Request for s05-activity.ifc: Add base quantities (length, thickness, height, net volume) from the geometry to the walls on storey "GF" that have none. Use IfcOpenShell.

First a look at what the model holds.

```python
import ifcopenshell
import ifcopenshell.util.element
import ifcopenshell.util.unit

model = ifcopenshell.open("s05-activity.ifc")
print(model.schema)
for unit_type in ("LENGTHUNIT", "AREAUNIT", "VOLUMEUNIT"):
    print(unit_type, ifcopenshell.util.unit.calculate_unit_scale(model, unit_type))
storey = next(s for s in model.by_type("IfcBuildingStorey") if s.Name == "GF")
walls = [e for e in ifcopenshell.util.element.get_decomposition(storey) if e.is_a("IfcWall")]
for e in sorted(walls, key=lambda e: e.id()):
    print(e.id(), e.is_a(), e.Name, list(ifcopenshell.util.element.get_psets(e, qtos_only=True)), sep=" | ")
```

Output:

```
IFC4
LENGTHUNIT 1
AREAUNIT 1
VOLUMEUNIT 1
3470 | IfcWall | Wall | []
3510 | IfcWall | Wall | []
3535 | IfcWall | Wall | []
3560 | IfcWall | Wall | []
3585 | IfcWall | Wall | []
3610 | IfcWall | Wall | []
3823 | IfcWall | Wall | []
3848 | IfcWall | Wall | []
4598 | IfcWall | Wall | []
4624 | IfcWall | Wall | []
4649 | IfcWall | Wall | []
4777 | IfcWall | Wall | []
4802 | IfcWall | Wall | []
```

```python
import ifcopenshell
import ifcopenshell.api.pset
import ifcopenshell.geom
import ifcopenshell.util.element
import ifcopenshell.util.shape
import ifcopenshell.util.unit

model = ifcopenshell.open("s05-activity.ifc")
unit_scale = ifcopenshell.util.unit.calculate_unit_scale(model)
volume_scale = ifcopenshell.util.unit.calculate_unit_scale(model, "VOLUMEUNIT")
settings = ifcopenshell.geom.settings()

storey = next(s for s in model.by_type("IfcBuildingStorey") if s.Name == "GF")
walls = [e for e in ifcopenshell.util.element.get_decomposition(storey) if e.is_a("IfcWall")]

for e in sorted(walls, key=lambda e: e.id()):
    if ifcopenshell.util.element.get_psets(e, qtos_only=True, should_inherit=False):
        continue
    # Geometry comes back in metres, in the element's own axes.
    shape = ifcopenshell.geom.create_shape(settings, e)
    values = {
        "Length": ifcopenshell.util.shape.get_x(shape.geometry) / unit_scale,
        "Width": ifcopenshell.util.shape.get_y(shape.geometry) / unit_scale,
        "Height": ifcopenshell.util.shape.get_z(shape.geometry) / unit_scale,
        "NetVolume": ifcopenshell.util.shape.get_volume(shape.geometry) / volume_scale,
    }
    qto = ifcopenshell.api.pset.add_qto(model, product=e, name="Qto_WallBaseQuantities")
    ifcopenshell.api.pset.edit_qto(model, qto=qto, properties=values)
    print(e.id(), {k: round(v, 3) for k, v in values.items()})

model.write("s05-activity_v2.ifc")
```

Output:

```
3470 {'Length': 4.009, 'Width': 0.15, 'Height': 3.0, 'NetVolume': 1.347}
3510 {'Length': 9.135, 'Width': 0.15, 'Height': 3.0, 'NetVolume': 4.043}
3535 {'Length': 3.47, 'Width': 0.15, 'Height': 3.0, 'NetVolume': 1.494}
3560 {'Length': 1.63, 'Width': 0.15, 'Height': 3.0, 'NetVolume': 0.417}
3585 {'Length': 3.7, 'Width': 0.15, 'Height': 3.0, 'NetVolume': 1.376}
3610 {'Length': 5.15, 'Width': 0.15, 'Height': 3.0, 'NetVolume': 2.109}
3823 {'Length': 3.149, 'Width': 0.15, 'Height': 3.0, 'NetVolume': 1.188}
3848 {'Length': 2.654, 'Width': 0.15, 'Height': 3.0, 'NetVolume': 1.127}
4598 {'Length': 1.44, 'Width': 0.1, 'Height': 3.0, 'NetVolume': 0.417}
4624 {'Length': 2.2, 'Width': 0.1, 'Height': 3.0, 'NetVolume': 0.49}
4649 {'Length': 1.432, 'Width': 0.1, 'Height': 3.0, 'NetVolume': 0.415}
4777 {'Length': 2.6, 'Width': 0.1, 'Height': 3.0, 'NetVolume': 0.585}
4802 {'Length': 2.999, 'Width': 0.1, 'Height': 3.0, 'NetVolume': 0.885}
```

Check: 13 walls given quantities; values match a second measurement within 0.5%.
